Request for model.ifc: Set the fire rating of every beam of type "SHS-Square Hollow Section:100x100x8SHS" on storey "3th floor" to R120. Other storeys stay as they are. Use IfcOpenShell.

First a look at what the model holds.

```python
import ifcopenshell
import ifcopenshell.util.element

model = ifcopenshell.open("model.ifc")
print(model.schema)
storey = next(s for s in model.by_type("IfcBuildingStorey") if s.Name == "3th floor")
beams = [e for e in ifcopenshell.util.element.get_decomposition(storey) if e.is_a("IfcBeam")]
seen = {}
for e in beams:
    element_type = ifcopenshell.util.element.get_type(e)
    key = (element_type.Name if element_type != e and element_type else None, ifcopenshell.util.element.get_pset(e, "Pset_BeamCommon", "FireRating"))
    seen[key] = seen.get(key, 0) + 1
for (name, value), count in sorted(seen.items(), key=str):
    print(count, "x", name, "|", value)
```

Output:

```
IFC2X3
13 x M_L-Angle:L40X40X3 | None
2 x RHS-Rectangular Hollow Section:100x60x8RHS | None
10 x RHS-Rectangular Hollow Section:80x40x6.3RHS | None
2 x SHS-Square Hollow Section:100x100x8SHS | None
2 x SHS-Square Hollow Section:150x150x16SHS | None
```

```python
import ifcopenshell
import ifcopenshell.api.pset
import ifcopenshell.util.element

model = ifcopenshell.open("model.ifc")

storey = next(s for s in model.by_type("IfcBuildingStorey") if s.Name == "3th floor")
beams = [e for e in ifcopenshell.util.element.get_decomposition(storey) if e.is_a("IfcBeam")]

count = 0
for e in beams:
    element_type = ifcopenshell.util.element.get_type(e)
    if element_type in (None, e) or element_type.Name != "SHS-Square Hollow Section:100x100x8SHS":
        continue
    # add_pset returns the element's existing set when there is one.
    pset = ifcopenshell.api.pset.add_pset(model, product=e, name="Pset_BeamCommon")
    ifcopenshell.api.pset.edit_pset(model, pset=pset, properties={"FireRating": "R120"})
    count += 1

print(count, "beams updated")

model.write("model_edited.ifc")
```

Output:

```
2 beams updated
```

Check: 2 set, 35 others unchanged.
